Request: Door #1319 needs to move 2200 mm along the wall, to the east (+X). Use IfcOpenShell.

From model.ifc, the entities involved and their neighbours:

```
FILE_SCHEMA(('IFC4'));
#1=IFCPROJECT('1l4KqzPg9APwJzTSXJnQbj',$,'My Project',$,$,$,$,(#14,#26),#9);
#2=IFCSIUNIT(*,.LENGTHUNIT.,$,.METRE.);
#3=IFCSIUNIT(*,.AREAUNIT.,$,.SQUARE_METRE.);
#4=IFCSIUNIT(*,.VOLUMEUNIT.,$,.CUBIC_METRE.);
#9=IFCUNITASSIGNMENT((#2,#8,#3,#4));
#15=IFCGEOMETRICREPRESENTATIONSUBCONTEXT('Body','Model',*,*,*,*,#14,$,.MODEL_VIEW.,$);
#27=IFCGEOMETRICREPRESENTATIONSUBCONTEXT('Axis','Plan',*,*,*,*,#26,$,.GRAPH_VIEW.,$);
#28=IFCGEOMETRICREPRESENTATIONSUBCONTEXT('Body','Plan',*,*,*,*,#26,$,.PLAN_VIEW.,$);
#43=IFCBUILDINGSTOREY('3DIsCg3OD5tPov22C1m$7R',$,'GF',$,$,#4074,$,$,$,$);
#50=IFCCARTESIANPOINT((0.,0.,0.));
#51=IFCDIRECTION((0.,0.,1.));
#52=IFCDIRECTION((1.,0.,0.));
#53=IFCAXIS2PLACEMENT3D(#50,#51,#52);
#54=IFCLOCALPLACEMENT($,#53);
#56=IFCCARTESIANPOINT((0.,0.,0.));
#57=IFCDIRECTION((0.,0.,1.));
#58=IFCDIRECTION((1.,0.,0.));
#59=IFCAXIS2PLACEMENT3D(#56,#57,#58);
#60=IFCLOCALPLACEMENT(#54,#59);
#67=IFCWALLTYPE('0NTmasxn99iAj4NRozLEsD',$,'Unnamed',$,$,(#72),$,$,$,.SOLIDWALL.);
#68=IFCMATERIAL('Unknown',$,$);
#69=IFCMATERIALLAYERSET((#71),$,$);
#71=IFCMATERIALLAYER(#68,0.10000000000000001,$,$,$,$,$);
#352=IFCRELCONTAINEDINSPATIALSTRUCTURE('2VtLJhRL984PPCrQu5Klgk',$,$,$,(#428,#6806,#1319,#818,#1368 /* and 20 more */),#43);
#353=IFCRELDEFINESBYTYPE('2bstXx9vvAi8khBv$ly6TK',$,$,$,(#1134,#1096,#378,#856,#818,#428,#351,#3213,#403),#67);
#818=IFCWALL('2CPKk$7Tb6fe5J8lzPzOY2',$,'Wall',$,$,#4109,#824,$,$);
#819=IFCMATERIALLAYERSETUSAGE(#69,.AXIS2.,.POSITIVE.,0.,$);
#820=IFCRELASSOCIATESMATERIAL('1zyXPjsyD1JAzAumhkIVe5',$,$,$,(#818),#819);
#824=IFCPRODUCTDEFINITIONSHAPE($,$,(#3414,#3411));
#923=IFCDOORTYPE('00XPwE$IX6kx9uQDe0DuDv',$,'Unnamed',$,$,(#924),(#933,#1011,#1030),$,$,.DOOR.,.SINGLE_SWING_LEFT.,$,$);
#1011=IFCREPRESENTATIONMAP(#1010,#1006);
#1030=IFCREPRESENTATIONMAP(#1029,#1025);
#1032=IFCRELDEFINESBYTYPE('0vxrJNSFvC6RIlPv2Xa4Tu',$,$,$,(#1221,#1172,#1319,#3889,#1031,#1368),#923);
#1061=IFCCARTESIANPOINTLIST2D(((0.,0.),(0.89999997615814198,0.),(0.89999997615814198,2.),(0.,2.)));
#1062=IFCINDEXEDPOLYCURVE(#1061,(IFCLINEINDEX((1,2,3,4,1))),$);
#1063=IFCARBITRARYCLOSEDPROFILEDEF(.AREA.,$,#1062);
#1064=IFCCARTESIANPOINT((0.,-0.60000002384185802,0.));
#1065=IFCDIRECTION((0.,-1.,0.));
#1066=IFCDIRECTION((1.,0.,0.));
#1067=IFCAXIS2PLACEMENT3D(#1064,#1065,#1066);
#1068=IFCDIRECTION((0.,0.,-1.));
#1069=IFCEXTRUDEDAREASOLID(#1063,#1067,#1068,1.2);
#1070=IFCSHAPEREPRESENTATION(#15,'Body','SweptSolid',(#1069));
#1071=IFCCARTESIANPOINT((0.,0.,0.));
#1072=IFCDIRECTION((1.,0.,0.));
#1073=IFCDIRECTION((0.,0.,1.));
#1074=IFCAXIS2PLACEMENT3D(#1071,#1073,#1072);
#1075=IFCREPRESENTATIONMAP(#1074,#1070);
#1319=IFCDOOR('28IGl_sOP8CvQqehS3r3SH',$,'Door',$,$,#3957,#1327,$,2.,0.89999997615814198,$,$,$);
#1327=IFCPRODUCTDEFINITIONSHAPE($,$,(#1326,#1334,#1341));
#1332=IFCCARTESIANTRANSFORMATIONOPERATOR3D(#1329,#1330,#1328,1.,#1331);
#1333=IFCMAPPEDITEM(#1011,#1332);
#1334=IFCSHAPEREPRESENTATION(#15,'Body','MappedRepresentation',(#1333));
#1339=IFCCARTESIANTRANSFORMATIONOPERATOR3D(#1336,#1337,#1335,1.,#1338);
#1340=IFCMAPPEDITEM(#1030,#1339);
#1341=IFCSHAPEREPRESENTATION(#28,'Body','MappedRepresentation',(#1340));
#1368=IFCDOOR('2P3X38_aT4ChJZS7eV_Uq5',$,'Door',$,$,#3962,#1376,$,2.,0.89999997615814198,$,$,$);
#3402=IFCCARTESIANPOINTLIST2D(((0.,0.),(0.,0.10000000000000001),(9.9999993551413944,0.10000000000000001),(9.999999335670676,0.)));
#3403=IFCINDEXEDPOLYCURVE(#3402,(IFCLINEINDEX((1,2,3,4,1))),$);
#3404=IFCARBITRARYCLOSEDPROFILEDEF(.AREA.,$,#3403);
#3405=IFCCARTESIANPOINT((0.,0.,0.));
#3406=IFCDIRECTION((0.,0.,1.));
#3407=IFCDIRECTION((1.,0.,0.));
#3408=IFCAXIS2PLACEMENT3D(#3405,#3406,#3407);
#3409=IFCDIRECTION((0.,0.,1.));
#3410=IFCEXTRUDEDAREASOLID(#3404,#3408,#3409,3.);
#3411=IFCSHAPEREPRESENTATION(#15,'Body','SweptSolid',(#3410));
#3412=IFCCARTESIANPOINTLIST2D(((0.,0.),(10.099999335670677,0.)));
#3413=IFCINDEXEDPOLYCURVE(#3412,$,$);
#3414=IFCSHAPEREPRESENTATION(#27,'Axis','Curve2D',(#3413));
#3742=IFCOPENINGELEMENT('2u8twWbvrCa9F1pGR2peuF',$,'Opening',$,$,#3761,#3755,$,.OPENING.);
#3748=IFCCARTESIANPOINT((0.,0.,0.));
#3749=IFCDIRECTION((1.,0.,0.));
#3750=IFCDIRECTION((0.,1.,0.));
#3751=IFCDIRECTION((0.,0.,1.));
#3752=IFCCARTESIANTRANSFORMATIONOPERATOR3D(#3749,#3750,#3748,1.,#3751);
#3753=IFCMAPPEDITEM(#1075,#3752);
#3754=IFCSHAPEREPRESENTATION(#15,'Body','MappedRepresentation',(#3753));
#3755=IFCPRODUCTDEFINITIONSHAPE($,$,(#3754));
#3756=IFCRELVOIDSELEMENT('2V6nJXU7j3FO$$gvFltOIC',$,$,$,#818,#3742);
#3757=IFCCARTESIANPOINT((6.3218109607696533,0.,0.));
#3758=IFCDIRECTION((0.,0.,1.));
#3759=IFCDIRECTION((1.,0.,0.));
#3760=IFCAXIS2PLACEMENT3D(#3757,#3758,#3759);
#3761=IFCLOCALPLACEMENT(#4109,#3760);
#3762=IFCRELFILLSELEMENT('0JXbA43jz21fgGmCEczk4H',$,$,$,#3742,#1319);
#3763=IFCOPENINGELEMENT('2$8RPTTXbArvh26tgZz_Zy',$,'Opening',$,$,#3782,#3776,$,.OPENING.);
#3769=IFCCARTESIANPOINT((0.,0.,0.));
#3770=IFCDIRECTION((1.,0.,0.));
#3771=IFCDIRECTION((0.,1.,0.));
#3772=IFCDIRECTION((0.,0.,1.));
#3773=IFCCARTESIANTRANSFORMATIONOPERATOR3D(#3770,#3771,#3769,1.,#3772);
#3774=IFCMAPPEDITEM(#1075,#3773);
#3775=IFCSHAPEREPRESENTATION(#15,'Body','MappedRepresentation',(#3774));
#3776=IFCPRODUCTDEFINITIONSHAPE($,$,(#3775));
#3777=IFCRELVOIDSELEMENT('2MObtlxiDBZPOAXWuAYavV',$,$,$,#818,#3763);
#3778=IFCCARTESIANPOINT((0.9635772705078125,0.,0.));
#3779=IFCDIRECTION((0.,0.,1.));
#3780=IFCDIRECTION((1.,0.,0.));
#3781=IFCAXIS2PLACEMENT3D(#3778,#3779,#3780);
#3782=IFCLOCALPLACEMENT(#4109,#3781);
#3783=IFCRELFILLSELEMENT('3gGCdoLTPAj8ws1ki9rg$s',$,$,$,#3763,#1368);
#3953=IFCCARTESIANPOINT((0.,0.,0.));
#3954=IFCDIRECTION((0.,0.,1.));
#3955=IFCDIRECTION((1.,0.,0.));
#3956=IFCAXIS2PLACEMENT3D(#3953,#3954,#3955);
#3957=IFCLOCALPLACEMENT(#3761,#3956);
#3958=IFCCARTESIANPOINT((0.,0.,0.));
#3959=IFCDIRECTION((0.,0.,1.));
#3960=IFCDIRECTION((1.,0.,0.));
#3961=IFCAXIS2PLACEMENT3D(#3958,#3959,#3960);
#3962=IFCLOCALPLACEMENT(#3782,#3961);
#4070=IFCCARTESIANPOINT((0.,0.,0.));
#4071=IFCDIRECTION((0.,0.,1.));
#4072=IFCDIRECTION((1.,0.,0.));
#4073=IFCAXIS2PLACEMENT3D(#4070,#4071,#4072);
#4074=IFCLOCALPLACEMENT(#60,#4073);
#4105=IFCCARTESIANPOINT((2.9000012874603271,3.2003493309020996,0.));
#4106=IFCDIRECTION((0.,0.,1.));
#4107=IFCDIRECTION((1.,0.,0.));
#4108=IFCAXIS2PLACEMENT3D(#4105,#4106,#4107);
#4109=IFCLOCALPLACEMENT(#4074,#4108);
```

```python
import ifcopenshell
import ifcopenshell.api.geometry
import ifcopenshell.util.placement
import ifcopenshell.util.unit

model = ifcopenshell.open("model.ifc")
unit_scale = ifcopenshell.util.unit.calculate_unit_scale(model)

door = model.by_guid("28IGl_sOP8CvQqehS3r3SH")
opening = door.FillsVoids[0].RelatingOpeningElement
wall = opening.VoidsElements[0].RelatingBuildingElement

wall_matrix = ifcopenshell.util.placement.get_local_placement(wall.ObjectPlacement)
shift = wall_matrix[:3, 0] * 2.2 / unit_scale
before = ifcopenshell.util.placement.get_local_placement(door.ObjectPlacement)[:3, 3].copy()

# The door is placed relative to its opening, so it follows when the opening moves.
matrix = ifcopenshell.util.placement.get_local_placement(opening.ObjectPlacement)
matrix[:3, 3] += shift
ifcopenshell.api.geometry.edit_object_placement(
    model, product=opening, matrix=matrix, is_si=False, should_transform_children=True
)

after = ifcopenshell.util.placement.get_local_placement(door.ObjectPlacement)[:3, 3]
print("door moved by", (after - before).round(3) + 0.0)

model.write("model-out.ifc")
```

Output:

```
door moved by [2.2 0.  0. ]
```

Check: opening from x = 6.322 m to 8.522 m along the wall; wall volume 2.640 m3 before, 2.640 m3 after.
